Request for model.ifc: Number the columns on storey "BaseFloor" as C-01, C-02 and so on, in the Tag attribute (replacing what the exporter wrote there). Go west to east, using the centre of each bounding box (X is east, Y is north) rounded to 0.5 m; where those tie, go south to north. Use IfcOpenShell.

First a look at what the model holds.

```python
import ifcopenshell
import ifcopenshell.util.element
import ifcopenshell.util.placement

model = ifcopenshell.open("model.ifc")
print(model.schema)
storey = next(s for s in model.by_type("IfcBuildingStorey") if s.Name == "BaseFloor")
columns = [e for e in ifcopenshell.util.element.get_decomposition(storey) if e.is_a("IfcColumn")]
for e in sorted(columns, key=lambda e: e.id()):
    origin = ifcopenshell.util.placement.get_local_placement(e.ObjectPlacement)[:3, 3]
    print(e.id(), e.Tag, e.Name, origin.round(2) + 0.0, sep=" | ")
```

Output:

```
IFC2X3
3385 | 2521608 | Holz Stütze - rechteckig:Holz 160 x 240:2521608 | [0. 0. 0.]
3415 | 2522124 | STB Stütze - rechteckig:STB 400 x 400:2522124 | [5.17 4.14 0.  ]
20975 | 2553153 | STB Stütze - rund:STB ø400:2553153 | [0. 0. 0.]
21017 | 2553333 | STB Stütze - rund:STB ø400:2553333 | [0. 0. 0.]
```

```python
import ifcopenshell
import ifcopenshell.geom
import ifcopenshell.util.element
import ifcopenshell.util.shape

model = ifcopenshell.open("model.ifc")
settings = ifcopenshell.geom.settings()
settings.set("use-world-coords", True)


def centre(element):
    shape = ifcopenshell.geom.create_shape(settings, element)
    return ifcopenshell.util.shape.get_bbox_centroid(shape.geometry)


storey = next(s for s in model.by_type("IfcBuildingStorey") if s.Name == "BaseFloor")
columns = [e for e in ifcopenshell.util.element.get_decomposition(storey) if e.is_a("IfcColumn")]

# Insertion points can sit at a corner or the storey origin, so sort by the geometry (in metres).
centres = {e: centre(e) for e in columns}
columns.sort(key=lambda e: (round(centres[e][0] / 0.5), centres[e][1]))

for i, e in enumerate(columns, start=1):
    number = f"C-{i:02d}"
    e.Tag = number
    print(e.id(), number)

model.write("model_v2.ifc")
```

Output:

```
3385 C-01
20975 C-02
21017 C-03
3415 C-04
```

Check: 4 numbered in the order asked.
